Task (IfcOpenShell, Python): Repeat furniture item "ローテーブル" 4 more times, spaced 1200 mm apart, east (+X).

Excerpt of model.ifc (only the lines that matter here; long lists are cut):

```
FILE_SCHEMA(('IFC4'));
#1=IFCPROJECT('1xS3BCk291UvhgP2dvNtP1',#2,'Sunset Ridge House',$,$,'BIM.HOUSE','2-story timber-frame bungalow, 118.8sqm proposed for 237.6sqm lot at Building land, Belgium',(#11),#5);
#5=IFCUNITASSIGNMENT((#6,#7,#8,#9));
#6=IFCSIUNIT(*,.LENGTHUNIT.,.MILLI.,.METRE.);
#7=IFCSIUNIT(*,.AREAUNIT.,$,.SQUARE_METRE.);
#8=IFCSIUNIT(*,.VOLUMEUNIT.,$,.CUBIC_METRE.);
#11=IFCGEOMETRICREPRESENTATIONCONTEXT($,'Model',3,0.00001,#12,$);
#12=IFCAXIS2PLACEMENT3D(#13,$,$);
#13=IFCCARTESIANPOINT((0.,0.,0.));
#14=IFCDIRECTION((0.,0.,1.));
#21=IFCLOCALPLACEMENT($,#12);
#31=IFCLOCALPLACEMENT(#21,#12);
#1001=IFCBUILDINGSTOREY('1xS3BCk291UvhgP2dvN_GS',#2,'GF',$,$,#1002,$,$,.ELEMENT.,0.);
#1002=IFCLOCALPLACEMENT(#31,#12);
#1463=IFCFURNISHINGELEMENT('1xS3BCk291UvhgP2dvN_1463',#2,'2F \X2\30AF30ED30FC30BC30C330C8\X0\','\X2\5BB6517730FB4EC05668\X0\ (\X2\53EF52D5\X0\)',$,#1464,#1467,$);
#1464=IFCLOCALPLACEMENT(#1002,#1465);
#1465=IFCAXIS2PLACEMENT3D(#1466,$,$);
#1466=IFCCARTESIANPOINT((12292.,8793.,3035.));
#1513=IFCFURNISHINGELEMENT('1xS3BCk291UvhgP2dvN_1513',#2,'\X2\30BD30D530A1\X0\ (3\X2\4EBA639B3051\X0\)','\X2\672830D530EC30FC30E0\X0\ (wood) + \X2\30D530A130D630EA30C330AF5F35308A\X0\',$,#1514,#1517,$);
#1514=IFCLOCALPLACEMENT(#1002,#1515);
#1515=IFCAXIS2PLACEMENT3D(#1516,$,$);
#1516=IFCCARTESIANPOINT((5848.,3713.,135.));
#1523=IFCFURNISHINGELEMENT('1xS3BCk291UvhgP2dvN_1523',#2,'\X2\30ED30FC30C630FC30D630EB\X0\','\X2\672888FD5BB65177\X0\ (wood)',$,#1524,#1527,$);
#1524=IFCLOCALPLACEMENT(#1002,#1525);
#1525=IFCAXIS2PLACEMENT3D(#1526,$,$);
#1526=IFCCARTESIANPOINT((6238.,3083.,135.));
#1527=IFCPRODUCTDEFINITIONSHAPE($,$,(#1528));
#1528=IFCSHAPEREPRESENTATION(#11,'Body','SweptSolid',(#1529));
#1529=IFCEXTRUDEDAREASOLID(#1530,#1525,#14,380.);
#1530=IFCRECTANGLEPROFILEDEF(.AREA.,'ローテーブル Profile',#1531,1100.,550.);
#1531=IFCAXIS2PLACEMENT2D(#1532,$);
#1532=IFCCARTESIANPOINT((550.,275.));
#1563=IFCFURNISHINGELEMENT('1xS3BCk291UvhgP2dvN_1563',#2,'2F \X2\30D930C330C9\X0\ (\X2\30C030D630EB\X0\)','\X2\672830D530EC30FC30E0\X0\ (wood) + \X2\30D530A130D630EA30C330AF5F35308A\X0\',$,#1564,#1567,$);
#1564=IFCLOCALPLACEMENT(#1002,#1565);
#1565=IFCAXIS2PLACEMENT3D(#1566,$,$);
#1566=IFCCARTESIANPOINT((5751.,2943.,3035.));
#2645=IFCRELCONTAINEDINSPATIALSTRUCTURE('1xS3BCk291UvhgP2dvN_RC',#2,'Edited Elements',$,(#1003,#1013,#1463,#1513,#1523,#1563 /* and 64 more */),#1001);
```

```python
import numpy as np
import ifcopenshell
import ifcopenshell.api.geometry
import ifcopenshell.api.root
import ifcopenshell.util.element
import ifcopenshell.util.placement
import ifcopenshell.util.unit

model = ifcopenshell.open("model.ifc")
unit_scale = ifcopenshell.util.unit.calculate_unit_scale(model)


def reuse_history(source, copy):
    """copy_class also copies each property set's owner history, people and application; keep the originals."""
    for rel in copy.IsDefinedBy:
        if rel.is_a("IfcRelDefinesByProperties") and (history := rel.RelatingPropertyDefinition.OwnerHistory):
            rel.RelatingPropertyDefinition.OwnerHistory = source.OwnerHistory
            ifcopenshell.util.element.remove_deep2(model, history)


source = model.by_guid("1xS3BCk291UvhgP2dvN_1523")
base = ifcopenshell.util.placement.get_local_placement(source.ObjectPlacement)
step = np.array([1.0, 0.0, 0.0]) * 1.2 / unit_scale

for i in range(1, 5):
    copy = ifcopenshell.api.root.copy_class(model, product=source)
    copy.Representation = ifcopenshell.util.element.copy_deep(
        model, source.Representation, exclude=["IfcGeometricRepresentationContext", "IfcRepresentationMap"]
    )
    reuse_history(source, copy)
    matrix = base.copy()
    matrix[:3, 3] += i * step
    print("added at", matrix[:3, 3].round(3) + 0.0)
    ifcopenshell.api.geometry.edit_object_placement(model, product=copy, matrix=matrix, is_si=False)

model.write("model_updated.ifc")
```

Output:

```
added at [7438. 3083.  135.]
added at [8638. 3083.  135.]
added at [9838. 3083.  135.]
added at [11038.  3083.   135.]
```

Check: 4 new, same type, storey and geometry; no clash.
